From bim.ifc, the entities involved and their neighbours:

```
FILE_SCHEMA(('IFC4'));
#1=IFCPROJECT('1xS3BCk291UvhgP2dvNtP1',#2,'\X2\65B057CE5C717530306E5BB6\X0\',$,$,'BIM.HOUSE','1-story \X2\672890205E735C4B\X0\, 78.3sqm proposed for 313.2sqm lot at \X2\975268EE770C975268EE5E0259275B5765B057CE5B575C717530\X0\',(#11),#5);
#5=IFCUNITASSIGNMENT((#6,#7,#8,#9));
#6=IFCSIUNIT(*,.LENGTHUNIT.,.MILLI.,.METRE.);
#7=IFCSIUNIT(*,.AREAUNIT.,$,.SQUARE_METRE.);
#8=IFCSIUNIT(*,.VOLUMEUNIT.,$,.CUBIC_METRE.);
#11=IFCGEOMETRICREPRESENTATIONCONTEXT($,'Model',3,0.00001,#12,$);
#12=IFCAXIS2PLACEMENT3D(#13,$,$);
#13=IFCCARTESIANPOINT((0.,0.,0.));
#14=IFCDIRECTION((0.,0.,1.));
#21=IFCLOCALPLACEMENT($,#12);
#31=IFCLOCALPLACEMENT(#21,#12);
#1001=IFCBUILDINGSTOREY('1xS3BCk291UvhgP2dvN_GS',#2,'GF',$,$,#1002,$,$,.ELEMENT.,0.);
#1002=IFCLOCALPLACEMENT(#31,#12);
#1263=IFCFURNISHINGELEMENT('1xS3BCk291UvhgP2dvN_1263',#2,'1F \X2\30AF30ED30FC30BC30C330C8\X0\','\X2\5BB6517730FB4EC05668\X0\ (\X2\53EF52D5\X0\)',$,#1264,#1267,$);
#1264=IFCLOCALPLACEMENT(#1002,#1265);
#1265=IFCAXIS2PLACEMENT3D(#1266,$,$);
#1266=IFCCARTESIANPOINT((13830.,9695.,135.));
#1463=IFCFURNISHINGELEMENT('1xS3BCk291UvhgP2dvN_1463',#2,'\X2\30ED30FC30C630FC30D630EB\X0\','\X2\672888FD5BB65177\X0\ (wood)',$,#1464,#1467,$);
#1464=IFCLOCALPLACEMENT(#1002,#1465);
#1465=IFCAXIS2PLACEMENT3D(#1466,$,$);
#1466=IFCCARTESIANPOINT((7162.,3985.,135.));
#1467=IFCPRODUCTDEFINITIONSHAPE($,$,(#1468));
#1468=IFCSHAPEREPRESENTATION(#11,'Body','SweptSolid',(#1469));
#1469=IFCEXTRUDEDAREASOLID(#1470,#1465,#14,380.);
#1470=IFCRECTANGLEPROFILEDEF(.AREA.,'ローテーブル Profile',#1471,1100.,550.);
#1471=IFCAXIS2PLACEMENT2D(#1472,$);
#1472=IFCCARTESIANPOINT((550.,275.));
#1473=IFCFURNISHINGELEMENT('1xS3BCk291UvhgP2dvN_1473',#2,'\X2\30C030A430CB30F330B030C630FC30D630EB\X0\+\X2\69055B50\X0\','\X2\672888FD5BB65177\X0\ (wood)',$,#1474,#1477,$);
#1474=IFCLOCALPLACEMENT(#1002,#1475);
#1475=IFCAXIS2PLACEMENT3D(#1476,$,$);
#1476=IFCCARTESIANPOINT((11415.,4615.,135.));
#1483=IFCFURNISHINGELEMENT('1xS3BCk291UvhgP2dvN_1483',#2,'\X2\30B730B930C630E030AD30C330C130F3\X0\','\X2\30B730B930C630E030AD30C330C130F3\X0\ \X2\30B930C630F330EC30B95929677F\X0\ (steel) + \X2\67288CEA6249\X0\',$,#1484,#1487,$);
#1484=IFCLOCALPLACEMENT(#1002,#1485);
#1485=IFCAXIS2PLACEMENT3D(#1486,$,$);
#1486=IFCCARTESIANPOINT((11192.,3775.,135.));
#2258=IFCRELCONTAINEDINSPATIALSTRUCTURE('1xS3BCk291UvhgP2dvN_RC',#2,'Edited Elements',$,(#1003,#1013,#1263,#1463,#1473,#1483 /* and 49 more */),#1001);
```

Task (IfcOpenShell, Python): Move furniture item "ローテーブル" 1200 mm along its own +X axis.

```python
import ifcopenshell
import ifcopenshell.api.geometry
import ifcopenshell.util.placement
import ifcopenshell.util.unit

model = ifcopenshell.open("bim.ifc")
unit_scale = ifcopenshell.util.unit.calculate_unit_scale(model)

item = model.by_id(1463)
matrix = ifcopenshell.util.placement.get_local_placement(item.ObjectPlacement)
matrix[:3, 3] += matrix[:3, 0] * 1.2 / unit_scale
ifcopenshell.api.geometry.edit_object_placement(model, product=item, matrix=matrix, is_si=False)

print(ifcopenshell.util.placement.get_local_placement(item.ObjectPlacement).round(3) + 0.0)

model.write("bim_rev.ifc")
```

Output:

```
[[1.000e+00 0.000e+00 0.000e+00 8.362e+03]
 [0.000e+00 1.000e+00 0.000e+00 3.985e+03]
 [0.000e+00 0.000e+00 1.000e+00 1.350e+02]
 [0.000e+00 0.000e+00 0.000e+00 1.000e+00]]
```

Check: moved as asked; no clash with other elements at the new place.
